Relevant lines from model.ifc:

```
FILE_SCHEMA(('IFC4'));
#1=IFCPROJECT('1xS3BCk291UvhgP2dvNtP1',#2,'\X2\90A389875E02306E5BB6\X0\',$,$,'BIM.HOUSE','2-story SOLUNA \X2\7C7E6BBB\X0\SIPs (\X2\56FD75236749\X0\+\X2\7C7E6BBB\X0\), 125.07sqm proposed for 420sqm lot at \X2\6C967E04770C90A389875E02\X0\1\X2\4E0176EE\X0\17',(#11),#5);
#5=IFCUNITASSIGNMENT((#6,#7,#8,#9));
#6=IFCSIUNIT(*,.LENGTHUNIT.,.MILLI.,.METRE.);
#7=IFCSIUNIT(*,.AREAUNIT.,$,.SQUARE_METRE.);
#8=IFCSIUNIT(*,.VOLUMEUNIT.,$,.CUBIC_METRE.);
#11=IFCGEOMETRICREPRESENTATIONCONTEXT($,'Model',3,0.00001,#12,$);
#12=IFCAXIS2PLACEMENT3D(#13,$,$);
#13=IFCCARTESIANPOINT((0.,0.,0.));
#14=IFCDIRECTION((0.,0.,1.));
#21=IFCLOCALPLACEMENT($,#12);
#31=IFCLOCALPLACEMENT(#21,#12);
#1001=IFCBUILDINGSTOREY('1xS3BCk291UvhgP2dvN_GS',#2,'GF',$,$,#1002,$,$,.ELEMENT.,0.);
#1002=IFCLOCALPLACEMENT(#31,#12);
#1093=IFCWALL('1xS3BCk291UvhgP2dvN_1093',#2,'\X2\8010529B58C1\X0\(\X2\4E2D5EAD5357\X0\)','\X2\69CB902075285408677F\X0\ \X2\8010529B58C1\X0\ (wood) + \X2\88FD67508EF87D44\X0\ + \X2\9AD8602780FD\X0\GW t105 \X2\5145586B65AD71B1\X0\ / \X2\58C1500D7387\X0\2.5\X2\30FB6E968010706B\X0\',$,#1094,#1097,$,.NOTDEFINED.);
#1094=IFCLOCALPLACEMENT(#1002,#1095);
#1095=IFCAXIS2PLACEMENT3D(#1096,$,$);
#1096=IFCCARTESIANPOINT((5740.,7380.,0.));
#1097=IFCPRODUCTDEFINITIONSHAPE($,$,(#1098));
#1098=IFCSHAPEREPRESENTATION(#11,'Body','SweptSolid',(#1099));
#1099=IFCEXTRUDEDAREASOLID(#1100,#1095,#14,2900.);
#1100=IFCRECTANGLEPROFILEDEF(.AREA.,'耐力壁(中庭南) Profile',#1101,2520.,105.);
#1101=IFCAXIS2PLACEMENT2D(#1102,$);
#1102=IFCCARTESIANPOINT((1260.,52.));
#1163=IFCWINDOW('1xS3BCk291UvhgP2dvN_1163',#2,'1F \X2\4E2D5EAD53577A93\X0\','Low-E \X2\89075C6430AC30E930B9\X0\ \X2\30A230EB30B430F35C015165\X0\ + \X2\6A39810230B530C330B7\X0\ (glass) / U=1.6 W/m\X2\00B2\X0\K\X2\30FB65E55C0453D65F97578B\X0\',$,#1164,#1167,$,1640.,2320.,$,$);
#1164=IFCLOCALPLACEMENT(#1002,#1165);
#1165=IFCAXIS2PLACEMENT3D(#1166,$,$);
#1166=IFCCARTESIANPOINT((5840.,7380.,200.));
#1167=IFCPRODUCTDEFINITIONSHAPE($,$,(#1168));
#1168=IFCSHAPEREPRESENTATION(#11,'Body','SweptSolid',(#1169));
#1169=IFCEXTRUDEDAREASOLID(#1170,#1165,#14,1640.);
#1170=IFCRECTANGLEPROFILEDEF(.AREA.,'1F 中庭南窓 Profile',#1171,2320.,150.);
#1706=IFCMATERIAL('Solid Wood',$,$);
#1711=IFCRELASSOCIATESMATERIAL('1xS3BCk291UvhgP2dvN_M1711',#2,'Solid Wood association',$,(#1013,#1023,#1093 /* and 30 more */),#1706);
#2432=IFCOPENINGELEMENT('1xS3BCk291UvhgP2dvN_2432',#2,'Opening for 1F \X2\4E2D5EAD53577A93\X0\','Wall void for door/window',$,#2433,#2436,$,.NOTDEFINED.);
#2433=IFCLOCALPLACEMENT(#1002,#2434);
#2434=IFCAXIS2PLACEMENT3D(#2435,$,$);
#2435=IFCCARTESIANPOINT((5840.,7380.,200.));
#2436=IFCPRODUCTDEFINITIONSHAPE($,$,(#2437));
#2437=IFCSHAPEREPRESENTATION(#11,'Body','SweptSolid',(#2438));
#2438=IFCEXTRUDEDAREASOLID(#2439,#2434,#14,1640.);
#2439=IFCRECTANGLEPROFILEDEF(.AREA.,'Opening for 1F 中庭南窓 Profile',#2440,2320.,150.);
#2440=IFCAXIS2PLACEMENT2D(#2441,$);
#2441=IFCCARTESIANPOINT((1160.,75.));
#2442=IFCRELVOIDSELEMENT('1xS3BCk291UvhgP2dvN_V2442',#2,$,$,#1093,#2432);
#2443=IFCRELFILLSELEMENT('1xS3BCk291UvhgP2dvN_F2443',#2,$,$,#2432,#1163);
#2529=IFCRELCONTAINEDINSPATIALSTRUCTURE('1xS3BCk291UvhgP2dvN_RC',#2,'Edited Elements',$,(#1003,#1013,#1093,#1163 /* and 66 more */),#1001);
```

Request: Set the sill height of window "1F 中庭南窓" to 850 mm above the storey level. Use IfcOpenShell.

```python
import numpy as np
import ifcopenshell
import ifcopenshell.api.geometry
import ifcopenshell.geom
import ifcopenshell.util.element
import ifcopenshell.util.placement
import ifcopenshell.util.shape
import ifcopenshell.util.unit

model = ifcopenshell.open("model.ifc")
unit_scale = ifcopenshell.util.unit.calculate_unit_scale(model)

window = model.by_guid("1xS3BCk291UvhgP2dvN_1163")
opening = window.FillsVoids[0].RelatingOpeningElement
storey = ifcopenshell.util.element.get_container(window, ifc_class="IfcBuildingStorey")
level = ifcopenshell.util.placement.get_local_placement(storey.ObjectPlacement)[2, 3]

# The opening's origin need not be at the sill, so measure its lowest point.
shape = ifcopenshell.geom.create_shape(ifcopenshell.geom.settings(), opening)
bottom = ifcopenshell.util.shape.get_shape_bottom_elevation(shape, shape.geometry) / unit_scale
dz = level + 850.0 - bottom

shift = np.array([0.0, 0.0, dz])
# The window is not placed relative to its opening, so move both.
for product in (opening, window):
    matrix = ifcopenshell.util.placement.get_local_placement(product.ObjectPlacement)
    matrix[:3, 3] += shift
    ifcopenshell.api.geometry.edit_object_placement(model, product=product, matrix=matrix, is_si=False)

print(f"moved by {dz * unit_scale:+.3f} m")

model.write("model-out.ifc")
```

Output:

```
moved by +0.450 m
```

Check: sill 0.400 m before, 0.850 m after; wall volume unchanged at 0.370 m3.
